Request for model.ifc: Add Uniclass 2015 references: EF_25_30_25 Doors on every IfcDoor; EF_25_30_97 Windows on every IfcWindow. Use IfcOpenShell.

First a look at what the model holds.

```python
import ifcopenshell

model = ifcopenshell.open("model.ifc")
print(model.schema)
print("classifications:", [c.Name for c in model.by_type("IfcClassification")])
for ifc_class in ("IfcDoor", "IfcRoof", "IfcStair", "IfcWall", "IfcWindow"):
    print(ifc_class, len(model.by_type(ifc_class)))
```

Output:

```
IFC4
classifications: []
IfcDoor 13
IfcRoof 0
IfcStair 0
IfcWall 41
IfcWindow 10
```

```python
import ifcopenshell
import ifcopenshell.api.classification

model = ifcopenshell.open("model.ifc")

system = ifcopenshell.api.classification.add_classification(model, classification="Uniclass 2015")

codes = {
    "IfcDoor": ("EF_25_30_25", "Doors"),
    "IfcWindow": ("EF_25_30_97", "Windows"),
}
for ifc_class, (code, name) in codes.items():
    products = model.by_type(ifc_class)
    ifcopenshell.api.classification.add_reference(
        model, products=products, classification=system, identification=code, name=name
    )
    print(code, len(products))

model.write("model_v2.ifc")
```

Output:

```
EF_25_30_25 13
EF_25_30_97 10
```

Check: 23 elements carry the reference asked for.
